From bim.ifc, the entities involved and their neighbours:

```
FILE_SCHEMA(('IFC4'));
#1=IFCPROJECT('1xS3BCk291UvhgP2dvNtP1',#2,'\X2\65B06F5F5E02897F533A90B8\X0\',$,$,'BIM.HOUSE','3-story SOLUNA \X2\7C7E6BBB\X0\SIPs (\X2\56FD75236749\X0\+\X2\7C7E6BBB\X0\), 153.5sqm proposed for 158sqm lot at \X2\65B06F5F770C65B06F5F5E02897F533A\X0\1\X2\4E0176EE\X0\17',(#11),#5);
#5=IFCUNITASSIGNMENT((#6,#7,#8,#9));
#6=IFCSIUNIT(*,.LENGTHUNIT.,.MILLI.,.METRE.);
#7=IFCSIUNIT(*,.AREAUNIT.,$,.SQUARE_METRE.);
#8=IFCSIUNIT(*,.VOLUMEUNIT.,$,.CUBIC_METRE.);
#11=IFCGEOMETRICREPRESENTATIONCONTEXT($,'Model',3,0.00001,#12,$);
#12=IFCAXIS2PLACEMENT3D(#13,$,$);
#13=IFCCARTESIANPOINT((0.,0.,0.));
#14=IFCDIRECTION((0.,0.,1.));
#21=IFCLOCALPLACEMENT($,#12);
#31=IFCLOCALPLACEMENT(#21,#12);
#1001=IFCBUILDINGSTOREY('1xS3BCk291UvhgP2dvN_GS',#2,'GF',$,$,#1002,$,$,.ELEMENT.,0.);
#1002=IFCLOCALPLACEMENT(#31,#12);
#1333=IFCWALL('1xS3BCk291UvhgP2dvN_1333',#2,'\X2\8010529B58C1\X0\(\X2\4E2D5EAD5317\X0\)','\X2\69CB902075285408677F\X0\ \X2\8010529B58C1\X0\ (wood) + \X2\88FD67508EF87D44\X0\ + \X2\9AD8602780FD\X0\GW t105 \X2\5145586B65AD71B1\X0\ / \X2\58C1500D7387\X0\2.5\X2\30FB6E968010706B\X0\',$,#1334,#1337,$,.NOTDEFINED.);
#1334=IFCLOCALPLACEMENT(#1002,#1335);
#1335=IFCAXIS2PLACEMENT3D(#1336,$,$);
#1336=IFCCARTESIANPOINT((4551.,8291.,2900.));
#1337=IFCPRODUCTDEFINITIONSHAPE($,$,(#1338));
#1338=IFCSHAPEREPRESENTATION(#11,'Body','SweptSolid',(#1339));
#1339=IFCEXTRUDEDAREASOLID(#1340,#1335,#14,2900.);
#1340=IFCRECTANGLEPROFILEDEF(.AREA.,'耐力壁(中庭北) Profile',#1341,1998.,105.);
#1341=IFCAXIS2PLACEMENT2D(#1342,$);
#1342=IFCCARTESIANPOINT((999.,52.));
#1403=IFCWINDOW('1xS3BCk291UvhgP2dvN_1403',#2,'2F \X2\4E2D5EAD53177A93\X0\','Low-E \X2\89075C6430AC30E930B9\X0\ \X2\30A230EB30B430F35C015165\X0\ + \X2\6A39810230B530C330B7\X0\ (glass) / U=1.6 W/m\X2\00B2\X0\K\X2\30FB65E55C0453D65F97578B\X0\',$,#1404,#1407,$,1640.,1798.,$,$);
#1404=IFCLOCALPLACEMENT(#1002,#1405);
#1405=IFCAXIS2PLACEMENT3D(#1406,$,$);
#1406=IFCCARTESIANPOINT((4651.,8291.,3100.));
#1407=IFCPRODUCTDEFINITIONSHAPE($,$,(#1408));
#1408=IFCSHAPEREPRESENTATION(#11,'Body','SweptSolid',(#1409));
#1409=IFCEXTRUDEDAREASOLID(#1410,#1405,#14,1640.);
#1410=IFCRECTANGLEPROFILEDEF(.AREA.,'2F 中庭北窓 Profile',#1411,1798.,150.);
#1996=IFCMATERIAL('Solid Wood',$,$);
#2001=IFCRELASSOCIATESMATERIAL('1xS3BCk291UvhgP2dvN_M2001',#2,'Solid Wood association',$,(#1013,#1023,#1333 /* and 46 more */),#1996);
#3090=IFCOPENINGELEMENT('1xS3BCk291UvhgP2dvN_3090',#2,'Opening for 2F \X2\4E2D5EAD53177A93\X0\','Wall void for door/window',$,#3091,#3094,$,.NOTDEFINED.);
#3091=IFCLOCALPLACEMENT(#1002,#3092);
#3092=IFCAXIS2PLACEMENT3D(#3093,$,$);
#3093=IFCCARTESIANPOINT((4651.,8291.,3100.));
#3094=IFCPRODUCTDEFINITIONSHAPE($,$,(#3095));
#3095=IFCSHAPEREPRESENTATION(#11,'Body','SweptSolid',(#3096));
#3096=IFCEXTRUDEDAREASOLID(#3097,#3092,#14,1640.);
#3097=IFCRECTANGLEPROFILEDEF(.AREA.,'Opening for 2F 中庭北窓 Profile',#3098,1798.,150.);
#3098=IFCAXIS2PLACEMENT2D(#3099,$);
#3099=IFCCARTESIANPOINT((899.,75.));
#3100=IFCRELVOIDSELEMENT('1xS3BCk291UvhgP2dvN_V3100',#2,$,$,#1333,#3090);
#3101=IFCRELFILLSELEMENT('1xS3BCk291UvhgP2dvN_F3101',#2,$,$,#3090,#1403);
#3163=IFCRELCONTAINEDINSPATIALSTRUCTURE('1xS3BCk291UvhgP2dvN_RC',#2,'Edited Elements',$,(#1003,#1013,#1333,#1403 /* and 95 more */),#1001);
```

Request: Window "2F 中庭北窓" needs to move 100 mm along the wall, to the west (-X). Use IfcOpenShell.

```python
import ifcopenshell
import ifcopenshell.api.geometry
import ifcopenshell.util.placement
import ifcopenshell.util.unit

model = ifcopenshell.open("bim.ifc")
unit_scale = ifcopenshell.util.unit.calculate_unit_scale(model)

window = model.by_id(1403)
opening = window.FillsVoids[0].RelatingOpeningElement
wall = opening.VoidsElements[0].RelatingBuildingElement

wall_matrix = ifcopenshell.util.placement.get_local_placement(wall.ObjectPlacement)
shift = wall_matrix[:3, 0] * -0.1 / unit_scale
before = ifcopenshell.util.placement.get_local_placement(window.ObjectPlacement)[:3, 3].copy()

# The window is not placed relative to its opening, so move both.
for product in (opening, window):
    matrix = ifcopenshell.util.placement.get_local_placement(product.ObjectPlacement)
    matrix[:3, 3] += shift
    ifcopenshell.api.geometry.edit_object_placement(model, product=product, matrix=matrix, is_si=False)

after = ifcopenshell.util.placement.get_local_placement(window.ObjectPlacement)[:3, 3]
print("window moved by", (after - before).round(3) + 0.0)

model.write("bim-out.ifc")
```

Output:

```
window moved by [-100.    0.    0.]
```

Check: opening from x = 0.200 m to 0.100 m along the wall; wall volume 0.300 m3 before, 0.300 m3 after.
